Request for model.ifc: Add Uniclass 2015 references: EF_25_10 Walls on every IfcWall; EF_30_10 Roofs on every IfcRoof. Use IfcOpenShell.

First a look at what the model holds.

```python
import ifcopenshell

model = ifcopenshell.open("model.ifc")
print(model.schema)
print("classifications:", [c.Name for c in model.by_type("IfcClassification")])
for ifc_class in ("IfcDoor", "IfcRoof", "IfcStair", "IfcWall", "IfcWindow"):
    print(ifc_class, len(model.by_type(ifc_class)))
```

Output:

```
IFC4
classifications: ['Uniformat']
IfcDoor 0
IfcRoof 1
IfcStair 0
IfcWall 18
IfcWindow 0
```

```python
import ifcopenshell
import ifcopenshell.api.classification

model = ifcopenshell.open("model.ifc")

system = ifcopenshell.api.classification.add_classification(model, classification="Uniclass 2015")

codes = {
    "IfcWall": ("EF_25_10", "Walls"),
    "IfcRoof": ("EF_30_10", "Roofs"),
}
for ifc_class, (code, name) in codes.items():
    products = model.by_type(ifc_class)
    ifcopenshell.api.classification.add_reference(
        model, products=products, classification=system, identification=code, name=name
    )
    print(code, len(products))

model.write("model_v2.ifc")
```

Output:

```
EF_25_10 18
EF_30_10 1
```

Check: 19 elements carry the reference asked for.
